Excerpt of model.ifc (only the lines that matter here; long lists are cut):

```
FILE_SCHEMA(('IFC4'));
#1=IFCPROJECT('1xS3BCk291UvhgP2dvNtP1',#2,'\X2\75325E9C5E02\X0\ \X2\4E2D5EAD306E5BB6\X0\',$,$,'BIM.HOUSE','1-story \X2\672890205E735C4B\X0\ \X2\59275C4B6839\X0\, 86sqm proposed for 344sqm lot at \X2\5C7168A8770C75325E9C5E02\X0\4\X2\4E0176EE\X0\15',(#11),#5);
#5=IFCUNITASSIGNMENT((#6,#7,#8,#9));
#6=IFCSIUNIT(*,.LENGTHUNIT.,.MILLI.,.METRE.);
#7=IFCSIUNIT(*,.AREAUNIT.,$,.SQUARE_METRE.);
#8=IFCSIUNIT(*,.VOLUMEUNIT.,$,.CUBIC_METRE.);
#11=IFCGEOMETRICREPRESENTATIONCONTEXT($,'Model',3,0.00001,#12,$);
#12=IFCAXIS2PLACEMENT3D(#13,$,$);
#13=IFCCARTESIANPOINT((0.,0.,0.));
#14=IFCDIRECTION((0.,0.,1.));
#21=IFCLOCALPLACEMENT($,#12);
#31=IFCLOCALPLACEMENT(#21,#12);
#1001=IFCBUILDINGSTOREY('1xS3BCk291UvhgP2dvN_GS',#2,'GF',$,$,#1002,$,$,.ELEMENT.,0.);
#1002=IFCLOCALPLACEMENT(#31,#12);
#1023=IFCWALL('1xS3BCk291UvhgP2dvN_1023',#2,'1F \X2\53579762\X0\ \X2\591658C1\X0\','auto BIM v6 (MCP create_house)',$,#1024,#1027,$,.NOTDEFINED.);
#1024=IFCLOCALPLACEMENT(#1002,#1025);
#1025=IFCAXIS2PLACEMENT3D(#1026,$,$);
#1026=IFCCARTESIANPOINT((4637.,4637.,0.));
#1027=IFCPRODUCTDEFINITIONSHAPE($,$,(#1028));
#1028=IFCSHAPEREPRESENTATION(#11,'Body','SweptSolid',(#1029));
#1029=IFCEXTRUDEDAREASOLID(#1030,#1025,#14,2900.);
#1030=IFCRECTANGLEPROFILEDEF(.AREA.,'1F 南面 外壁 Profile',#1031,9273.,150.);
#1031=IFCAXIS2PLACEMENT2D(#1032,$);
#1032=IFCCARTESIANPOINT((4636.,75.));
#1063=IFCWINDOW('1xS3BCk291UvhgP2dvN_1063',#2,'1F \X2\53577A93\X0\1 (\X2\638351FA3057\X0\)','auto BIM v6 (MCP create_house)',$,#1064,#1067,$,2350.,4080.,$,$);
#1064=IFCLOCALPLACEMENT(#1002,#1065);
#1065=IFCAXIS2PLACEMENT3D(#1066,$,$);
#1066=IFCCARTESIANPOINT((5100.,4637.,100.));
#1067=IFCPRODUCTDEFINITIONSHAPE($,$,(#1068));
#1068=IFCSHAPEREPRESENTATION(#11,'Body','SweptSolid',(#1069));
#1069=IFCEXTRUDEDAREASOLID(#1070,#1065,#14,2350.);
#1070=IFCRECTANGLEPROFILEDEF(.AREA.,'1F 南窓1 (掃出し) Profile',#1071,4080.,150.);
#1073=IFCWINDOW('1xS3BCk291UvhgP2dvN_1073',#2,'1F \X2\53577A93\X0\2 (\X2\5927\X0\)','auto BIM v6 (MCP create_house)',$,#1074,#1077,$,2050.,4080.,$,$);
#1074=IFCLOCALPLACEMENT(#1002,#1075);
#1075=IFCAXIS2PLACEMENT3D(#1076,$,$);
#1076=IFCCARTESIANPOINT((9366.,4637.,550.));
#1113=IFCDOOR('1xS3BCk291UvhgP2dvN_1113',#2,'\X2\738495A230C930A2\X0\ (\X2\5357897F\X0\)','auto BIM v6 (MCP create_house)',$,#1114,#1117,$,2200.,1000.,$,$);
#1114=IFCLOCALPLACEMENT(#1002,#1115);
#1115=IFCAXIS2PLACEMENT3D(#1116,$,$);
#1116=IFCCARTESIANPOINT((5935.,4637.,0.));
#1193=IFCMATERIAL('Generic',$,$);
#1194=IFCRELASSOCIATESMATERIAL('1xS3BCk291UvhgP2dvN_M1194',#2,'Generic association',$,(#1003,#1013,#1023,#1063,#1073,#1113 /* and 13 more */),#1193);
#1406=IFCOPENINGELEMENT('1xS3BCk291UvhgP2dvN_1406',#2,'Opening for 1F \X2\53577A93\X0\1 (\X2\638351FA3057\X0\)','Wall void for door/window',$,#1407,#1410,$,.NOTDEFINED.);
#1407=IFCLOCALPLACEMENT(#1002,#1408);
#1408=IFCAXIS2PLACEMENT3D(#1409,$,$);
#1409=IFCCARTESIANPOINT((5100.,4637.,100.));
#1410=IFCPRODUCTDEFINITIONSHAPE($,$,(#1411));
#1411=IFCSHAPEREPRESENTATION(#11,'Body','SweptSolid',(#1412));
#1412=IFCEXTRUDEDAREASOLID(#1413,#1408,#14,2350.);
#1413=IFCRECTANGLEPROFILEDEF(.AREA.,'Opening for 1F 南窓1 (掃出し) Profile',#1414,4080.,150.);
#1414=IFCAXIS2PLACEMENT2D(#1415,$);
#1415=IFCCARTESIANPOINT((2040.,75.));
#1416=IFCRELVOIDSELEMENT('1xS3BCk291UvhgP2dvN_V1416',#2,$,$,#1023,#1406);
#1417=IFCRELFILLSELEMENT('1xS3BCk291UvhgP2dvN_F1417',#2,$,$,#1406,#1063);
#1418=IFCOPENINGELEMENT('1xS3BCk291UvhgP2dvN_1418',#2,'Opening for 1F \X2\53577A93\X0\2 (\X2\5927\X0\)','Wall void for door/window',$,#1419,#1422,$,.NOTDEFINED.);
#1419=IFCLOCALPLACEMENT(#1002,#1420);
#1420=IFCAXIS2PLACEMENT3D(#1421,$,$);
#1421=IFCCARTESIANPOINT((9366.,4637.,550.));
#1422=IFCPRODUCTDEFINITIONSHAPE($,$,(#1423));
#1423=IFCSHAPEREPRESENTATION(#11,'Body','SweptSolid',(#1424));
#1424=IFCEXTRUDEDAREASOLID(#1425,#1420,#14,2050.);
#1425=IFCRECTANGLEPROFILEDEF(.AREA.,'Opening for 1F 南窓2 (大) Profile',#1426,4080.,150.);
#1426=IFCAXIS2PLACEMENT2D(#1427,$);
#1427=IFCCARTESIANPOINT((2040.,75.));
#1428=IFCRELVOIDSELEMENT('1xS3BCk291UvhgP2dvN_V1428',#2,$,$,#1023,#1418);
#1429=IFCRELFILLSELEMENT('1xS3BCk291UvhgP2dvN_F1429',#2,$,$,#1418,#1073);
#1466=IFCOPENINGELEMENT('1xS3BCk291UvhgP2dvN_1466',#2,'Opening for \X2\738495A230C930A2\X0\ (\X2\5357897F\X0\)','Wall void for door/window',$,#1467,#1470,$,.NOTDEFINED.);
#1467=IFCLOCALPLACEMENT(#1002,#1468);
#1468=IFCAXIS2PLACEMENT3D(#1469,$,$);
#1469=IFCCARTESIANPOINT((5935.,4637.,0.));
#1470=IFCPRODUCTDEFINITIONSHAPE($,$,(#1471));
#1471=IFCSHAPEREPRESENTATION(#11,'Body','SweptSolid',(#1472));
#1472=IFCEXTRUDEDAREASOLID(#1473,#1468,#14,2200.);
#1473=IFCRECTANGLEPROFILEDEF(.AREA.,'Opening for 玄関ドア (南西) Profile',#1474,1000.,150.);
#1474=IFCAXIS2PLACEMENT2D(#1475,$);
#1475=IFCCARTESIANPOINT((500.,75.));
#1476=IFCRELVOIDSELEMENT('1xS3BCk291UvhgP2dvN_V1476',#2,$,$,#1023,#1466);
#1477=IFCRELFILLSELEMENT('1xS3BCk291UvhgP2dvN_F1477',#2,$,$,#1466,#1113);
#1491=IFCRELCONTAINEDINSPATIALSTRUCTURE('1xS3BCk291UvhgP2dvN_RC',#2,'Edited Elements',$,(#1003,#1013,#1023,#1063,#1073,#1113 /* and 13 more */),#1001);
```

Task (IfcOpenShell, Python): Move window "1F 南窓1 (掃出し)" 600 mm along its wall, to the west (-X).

```python
import ifcopenshell
import ifcopenshell.api.geometry
import ifcopenshell.util.placement

model = ifcopenshell.open("model.ifc")

window = model.by_guid("1xS3BCk291UvhgP2dvN_1063")
opening = window.FillsVoids[0].RelatingOpeningElement
wall = opening.VoidsElements[0].RelatingBuildingElement

wall_matrix = ifcopenshell.util.placement.get_local_placement(wall.ObjectPlacement)
shift = wall_matrix[:3, 0] * -600.0
before = ifcopenshell.util.placement.get_local_placement(window.ObjectPlacement)[:3, 3].copy()

# The window is not placed relative to its opening, so move both.
for product in (opening, window):
    matrix = ifcopenshell.util.placement.get_local_placement(product.ObjectPlacement)
    matrix[:3, 3] += shift
    ifcopenshell.api.geometry.edit_object_placement(model, product=product, matrix=matrix, is_si=False)

after = ifcopenshell.util.placement.get_local_placement(window.ObjectPlacement)[:3, 3]
print("window moved by", (after - before).round(3) + 0.0)

model.write("model_rev.ifc")
```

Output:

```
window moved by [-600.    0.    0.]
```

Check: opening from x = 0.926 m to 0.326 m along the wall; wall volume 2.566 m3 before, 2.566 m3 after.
